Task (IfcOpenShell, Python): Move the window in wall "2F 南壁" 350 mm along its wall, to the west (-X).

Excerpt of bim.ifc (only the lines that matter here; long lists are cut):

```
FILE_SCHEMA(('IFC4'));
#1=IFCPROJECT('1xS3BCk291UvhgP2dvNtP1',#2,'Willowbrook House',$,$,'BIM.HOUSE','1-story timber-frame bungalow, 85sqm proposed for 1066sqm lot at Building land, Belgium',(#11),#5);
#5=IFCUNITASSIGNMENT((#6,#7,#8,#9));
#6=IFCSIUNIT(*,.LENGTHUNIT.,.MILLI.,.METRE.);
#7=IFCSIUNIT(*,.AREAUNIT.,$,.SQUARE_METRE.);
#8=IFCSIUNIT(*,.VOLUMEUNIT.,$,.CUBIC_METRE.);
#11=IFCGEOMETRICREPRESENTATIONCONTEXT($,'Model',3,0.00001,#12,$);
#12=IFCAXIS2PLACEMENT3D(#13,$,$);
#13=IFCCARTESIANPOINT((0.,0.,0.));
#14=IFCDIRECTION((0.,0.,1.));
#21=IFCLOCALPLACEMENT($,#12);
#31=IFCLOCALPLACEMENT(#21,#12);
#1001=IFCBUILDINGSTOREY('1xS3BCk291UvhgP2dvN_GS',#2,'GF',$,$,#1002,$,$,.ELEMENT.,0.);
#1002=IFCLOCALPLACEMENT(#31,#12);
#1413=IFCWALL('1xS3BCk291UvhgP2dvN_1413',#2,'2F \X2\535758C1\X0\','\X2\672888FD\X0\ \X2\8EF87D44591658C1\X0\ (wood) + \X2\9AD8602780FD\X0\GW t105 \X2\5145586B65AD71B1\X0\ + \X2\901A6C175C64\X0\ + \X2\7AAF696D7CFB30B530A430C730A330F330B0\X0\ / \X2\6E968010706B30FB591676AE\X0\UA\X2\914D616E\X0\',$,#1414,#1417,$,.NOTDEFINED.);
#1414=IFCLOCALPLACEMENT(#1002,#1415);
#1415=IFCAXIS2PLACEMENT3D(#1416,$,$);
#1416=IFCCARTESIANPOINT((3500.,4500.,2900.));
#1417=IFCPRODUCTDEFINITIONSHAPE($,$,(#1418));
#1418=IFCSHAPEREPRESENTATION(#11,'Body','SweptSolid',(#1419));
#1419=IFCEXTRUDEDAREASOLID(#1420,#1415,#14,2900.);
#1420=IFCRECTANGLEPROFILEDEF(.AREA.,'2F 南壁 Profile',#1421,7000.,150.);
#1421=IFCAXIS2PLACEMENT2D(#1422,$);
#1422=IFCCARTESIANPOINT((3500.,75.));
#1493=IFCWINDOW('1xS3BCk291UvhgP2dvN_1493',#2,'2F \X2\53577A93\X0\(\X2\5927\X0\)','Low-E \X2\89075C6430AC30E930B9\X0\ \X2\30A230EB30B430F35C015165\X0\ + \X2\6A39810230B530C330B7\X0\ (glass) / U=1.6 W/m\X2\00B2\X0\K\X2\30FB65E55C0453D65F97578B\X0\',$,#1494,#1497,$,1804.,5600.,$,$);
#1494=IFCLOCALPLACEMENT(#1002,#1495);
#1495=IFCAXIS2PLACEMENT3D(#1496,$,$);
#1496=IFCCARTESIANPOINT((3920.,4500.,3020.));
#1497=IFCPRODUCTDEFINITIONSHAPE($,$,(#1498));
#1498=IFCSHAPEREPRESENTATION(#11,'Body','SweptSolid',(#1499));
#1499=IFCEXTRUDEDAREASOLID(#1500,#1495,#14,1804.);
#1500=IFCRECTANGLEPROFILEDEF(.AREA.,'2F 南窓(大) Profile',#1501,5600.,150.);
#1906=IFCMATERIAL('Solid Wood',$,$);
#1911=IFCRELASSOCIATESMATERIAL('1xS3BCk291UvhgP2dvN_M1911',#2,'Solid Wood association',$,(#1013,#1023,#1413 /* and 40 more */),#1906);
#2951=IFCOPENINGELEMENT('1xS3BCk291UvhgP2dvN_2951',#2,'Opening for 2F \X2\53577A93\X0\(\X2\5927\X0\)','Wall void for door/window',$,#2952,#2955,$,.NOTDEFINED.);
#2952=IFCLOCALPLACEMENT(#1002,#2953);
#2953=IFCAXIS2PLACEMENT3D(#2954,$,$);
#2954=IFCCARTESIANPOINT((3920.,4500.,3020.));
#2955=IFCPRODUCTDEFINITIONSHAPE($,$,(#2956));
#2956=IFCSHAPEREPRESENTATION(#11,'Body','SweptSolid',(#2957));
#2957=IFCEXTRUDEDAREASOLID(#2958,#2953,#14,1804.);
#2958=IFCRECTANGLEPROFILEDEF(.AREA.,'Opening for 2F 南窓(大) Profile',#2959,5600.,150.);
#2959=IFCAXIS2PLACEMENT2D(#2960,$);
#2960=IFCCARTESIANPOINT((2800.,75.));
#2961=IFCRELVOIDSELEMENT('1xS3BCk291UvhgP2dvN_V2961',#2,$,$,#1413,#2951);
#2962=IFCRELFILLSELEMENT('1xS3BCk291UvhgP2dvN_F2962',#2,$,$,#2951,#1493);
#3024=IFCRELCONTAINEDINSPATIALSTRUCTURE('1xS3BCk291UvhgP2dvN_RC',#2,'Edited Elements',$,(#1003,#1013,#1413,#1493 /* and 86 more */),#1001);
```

```python
import ifcopenshell
import ifcopenshell.api.geometry
import ifcopenshell.util.placement
import ifcopenshell.util.unit

model = ifcopenshell.open("bim.ifc")
unit_scale = ifcopenshell.util.unit.calculate_unit_scale(model)

window = model.by_guid("1xS3BCk291UvhgP2dvN_1493")
opening = window.FillsVoids[0].RelatingOpeningElement
wall = opening.VoidsElements[0].RelatingBuildingElement

wall_matrix = ifcopenshell.util.placement.get_local_placement(wall.ObjectPlacement)
shift = wall_matrix[:3, 0] * -0.35 / unit_scale
before = ifcopenshell.util.placement.get_local_placement(window.ObjectPlacement)[:3, 3].copy()

# The window is not placed relative to its opening, so move both.
for product in (opening, window):
    matrix = ifcopenshell.util.placement.get_local_placement(product.ObjectPlacement)
    matrix[:3, 3] += shift
    ifcopenshell.api.geometry.edit_object_placement(model, product=product, matrix=matrix, is_si=False)

after = ifcopenshell.util.placement.get_local_placement(window.ObjectPlacement)[:3, 3]
print("window moved by", (after - before).round(3) + 0.0)

model.write("bim-out.ifc")
```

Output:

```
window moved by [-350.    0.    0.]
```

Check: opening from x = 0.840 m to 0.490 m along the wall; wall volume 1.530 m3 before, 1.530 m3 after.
